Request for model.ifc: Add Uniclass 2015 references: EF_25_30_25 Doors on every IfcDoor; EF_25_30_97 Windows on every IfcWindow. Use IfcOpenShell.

First a look at what the model holds.

```python
import ifcopenshell

model = ifcopenshell.open("model.ifc")
print(model.schema)
print("classifications:", [c.Name for c in model.by_type("IfcClassification")])
for ifc_class in ("IfcDoor", "IfcRoof", "IfcStair", "IfcWall", "IfcWindow"):
    print(ifc_class, len(model.by_type(ifc_class)))
```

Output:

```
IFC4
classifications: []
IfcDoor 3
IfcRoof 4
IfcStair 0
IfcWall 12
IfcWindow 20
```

```python
import ifcopenshell
import ifcopenshell.api.classification

model = ifcopenshell.open("model.ifc")

system = ifcopenshell.api.classification.add_classification(model, classification="Uniclass 2015")

codes = {
    "IfcDoor": ("EF_25_30_25", "Doors"),
    "IfcWindow": ("EF_25_30_97", "Windows"),
}
for ifc_class, (code, name) in codes.items():
    products = model.by_type(ifc_class)
    ifcopenshell.api.classification.add_reference(
        model, products=products, classification=system, identification=code, name=name
    )
    print(code, len(products))

model.write("model_updated.ifc")
```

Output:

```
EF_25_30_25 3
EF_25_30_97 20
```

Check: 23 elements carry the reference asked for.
